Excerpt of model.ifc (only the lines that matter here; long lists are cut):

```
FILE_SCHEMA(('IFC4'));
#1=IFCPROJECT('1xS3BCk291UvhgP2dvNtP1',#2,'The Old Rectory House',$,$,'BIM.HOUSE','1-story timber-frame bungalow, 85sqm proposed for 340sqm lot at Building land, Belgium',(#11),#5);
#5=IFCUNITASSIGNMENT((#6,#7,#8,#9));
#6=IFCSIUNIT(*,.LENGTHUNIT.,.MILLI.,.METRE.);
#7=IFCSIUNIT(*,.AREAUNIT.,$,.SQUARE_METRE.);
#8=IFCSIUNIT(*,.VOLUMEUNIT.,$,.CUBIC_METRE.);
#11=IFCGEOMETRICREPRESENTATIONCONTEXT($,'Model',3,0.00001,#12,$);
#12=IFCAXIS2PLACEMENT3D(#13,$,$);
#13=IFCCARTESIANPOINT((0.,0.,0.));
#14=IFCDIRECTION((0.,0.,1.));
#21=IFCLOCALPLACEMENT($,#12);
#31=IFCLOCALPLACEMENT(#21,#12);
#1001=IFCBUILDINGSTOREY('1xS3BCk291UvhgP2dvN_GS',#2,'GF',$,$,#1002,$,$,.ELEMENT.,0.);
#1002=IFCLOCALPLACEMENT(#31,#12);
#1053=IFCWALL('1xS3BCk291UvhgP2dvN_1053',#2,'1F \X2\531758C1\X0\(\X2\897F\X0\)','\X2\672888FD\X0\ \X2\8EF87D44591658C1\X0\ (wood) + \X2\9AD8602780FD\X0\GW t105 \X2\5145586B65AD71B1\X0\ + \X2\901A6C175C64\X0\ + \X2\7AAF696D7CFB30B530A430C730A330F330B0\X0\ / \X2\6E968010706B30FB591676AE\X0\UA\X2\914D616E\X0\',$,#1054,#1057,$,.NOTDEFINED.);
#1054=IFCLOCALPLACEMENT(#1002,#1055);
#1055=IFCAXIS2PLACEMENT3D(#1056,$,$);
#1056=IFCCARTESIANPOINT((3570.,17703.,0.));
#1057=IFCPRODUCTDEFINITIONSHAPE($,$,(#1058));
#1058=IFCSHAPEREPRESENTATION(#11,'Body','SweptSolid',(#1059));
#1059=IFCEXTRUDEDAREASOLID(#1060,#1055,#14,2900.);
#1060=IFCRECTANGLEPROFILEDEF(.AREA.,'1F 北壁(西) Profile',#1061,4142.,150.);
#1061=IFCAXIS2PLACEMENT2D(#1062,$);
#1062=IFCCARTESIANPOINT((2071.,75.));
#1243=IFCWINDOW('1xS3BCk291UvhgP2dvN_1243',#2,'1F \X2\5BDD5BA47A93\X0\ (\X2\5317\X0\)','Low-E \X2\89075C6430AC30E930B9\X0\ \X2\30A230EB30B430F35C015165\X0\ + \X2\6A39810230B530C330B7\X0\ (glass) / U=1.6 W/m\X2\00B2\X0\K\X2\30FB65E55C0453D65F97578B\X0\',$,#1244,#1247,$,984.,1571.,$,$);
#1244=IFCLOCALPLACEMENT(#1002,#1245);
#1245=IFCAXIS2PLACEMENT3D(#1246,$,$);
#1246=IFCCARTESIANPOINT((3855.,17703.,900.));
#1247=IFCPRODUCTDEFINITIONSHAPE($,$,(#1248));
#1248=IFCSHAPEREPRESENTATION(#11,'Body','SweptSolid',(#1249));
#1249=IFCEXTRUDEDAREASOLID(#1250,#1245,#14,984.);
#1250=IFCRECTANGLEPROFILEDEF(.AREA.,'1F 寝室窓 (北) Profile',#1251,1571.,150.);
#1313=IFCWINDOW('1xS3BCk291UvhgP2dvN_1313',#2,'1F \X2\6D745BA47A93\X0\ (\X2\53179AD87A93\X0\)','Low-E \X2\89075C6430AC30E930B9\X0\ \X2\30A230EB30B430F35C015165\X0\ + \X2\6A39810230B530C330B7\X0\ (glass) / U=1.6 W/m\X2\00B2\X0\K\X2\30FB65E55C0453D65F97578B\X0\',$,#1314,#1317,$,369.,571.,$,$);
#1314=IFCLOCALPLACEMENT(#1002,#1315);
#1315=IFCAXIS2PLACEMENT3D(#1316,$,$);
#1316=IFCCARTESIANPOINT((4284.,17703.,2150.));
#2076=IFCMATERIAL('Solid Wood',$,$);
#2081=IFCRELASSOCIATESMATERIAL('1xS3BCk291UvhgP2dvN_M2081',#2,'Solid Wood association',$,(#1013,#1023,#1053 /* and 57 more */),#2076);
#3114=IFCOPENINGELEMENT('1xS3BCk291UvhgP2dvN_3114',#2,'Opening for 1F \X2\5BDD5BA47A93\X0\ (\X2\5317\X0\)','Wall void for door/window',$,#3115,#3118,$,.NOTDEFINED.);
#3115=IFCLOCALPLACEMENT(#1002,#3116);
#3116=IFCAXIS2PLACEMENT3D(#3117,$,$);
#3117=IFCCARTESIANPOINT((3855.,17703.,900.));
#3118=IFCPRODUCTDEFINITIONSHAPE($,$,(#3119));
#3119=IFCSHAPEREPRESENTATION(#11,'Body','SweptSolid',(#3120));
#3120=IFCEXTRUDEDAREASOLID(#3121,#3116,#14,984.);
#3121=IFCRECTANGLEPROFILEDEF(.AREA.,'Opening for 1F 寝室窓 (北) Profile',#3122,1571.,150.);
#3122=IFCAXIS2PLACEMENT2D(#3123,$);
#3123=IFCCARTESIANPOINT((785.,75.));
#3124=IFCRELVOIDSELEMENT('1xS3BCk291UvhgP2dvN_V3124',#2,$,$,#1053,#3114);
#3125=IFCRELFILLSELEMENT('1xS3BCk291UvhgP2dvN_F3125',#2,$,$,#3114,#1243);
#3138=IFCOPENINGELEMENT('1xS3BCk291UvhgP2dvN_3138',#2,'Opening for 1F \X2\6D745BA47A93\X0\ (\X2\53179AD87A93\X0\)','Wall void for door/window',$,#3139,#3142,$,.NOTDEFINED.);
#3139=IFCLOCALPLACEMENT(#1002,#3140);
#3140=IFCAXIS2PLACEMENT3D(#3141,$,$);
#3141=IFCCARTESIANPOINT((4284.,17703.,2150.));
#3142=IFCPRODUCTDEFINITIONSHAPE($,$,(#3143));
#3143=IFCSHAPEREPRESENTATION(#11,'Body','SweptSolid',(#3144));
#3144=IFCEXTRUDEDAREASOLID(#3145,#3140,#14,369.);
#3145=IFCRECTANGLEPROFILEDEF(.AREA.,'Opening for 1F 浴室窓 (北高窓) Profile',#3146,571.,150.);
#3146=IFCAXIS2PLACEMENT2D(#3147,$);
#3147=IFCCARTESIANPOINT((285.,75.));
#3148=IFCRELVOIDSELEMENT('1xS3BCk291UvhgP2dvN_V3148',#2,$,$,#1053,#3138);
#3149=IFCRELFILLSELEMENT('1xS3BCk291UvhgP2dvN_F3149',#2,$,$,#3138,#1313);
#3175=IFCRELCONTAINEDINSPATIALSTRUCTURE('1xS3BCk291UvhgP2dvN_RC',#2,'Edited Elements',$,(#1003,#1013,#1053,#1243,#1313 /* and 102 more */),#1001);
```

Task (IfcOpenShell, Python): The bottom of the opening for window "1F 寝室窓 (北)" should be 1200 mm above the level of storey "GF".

```python
import numpy as np
import ifcopenshell
import ifcopenshell.api.geometry
import ifcopenshell.geom
import ifcopenshell.util.element
import ifcopenshell.util.placement
import ifcopenshell.util.shape
import ifcopenshell.util.unit

model = ifcopenshell.open("model.ifc")
unit_scale = ifcopenshell.util.unit.calculate_unit_scale(model)

window = model.by_id(1243)
opening = window.FillsVoids[0].RelatingOpeningElement
storey = ifcopenshell.util.element.get_container(window, ifc_class="IfcBuildingStorey")
level = ifcopenshell.util.placement.get_local_placement(storey.ObjectPlacement)[2, 3]

# The opening's origin need not be at the sill, so measure its lowest point.
shape = ifcopenshell.geom.create_shape(ifcopenshell.geom.settings(), opening)
bottom = ifcopenshell.util.shape.get_shape_bottom_elevation(shape, shape.geometry) / unit_scale
dz = level + 1.2 / unit_scale - bottom

shift = np.array([0.0, 0.0, dz])
# The window is not placed relative to its opening, so move both.
for product in (opening, window):
    matrix = ifcopenshell.util.placement.get_local_placement(product.ObjectPlacement)
    matrix[:3, 3] += shift
    ifcopenshell.api.geometry.edit_object_placement(model, product=product, matrix=matrix, is_si=False)

print(f"moved by {dz * unit_scale:+.3f} m")

model.write("model-out.ifc")
```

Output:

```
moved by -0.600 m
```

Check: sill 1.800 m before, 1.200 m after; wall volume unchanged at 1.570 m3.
